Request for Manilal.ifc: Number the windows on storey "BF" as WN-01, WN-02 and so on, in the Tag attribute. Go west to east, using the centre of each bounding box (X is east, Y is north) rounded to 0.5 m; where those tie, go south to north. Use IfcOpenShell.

First a look at what the model holds.

```python
import ifcopenshell
import ifcopenshell.util.element
import ifcopenshell.util.placement

model = ifcopenshell.open("Manilal.ifc")
print(model.schema)
storey = next(s for s in model.by_type("IfcBuildingStorey") if s.Name == "BF")
windows = [e for e in ifcopenshell.util.element.get_decomposition(storey) if e.is_a("IfcWindow")]
for e in sorted(windows, key=lambda e: e.id()):
    origin = ifcopenshell.util.placement.get_local_placement(e.ObjectPlacement)[:3, 3]
    print(e.id(), e.Tag, e.Name, origin.round(2) + 0.0, sep=" | ")
```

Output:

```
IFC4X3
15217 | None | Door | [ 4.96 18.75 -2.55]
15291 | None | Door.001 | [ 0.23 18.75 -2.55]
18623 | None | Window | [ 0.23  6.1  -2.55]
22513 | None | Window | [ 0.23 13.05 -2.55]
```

```python
import ifcopenshell
import ifcopenshell.geom
import ifcopenshell.util.element
import ifcopenshell.util.shape

model = ifcopenshell.open("Manilal.ifc")
settings = ifcopenshell.geom.settings()
settings.set("use-world-coords", True)


def centre(element):
    shape = ifcopenshell.geom.create_shape(settings, element)
    return ifcopenshell.util.shape.get_bbox_centroid(shape.geometry)


storey = next(s for s in model.by_type("IfcBuildingStorey") if s.Name == "BF")
windows = [e for e in ifcopenshell.util.element.get_decomposition(storey) if e.is_a("IfcWindow")]

# Insertion points can sit at a corner or the storey origin, so sort by the geometry (in metres).
centres = {e: centre(e) for e in windows}
windows.sort(key=lambda e: (round(centres[e][0] / 0.5), centres[e][1]))

for i, e in enumerate(windows, start=1):
    number = f"WN-{i:02d}"
    e.Tag = number
    print(e.id(), number)

model.write("Manilal-out.ifc")
```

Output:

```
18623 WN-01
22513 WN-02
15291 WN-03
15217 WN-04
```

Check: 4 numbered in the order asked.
